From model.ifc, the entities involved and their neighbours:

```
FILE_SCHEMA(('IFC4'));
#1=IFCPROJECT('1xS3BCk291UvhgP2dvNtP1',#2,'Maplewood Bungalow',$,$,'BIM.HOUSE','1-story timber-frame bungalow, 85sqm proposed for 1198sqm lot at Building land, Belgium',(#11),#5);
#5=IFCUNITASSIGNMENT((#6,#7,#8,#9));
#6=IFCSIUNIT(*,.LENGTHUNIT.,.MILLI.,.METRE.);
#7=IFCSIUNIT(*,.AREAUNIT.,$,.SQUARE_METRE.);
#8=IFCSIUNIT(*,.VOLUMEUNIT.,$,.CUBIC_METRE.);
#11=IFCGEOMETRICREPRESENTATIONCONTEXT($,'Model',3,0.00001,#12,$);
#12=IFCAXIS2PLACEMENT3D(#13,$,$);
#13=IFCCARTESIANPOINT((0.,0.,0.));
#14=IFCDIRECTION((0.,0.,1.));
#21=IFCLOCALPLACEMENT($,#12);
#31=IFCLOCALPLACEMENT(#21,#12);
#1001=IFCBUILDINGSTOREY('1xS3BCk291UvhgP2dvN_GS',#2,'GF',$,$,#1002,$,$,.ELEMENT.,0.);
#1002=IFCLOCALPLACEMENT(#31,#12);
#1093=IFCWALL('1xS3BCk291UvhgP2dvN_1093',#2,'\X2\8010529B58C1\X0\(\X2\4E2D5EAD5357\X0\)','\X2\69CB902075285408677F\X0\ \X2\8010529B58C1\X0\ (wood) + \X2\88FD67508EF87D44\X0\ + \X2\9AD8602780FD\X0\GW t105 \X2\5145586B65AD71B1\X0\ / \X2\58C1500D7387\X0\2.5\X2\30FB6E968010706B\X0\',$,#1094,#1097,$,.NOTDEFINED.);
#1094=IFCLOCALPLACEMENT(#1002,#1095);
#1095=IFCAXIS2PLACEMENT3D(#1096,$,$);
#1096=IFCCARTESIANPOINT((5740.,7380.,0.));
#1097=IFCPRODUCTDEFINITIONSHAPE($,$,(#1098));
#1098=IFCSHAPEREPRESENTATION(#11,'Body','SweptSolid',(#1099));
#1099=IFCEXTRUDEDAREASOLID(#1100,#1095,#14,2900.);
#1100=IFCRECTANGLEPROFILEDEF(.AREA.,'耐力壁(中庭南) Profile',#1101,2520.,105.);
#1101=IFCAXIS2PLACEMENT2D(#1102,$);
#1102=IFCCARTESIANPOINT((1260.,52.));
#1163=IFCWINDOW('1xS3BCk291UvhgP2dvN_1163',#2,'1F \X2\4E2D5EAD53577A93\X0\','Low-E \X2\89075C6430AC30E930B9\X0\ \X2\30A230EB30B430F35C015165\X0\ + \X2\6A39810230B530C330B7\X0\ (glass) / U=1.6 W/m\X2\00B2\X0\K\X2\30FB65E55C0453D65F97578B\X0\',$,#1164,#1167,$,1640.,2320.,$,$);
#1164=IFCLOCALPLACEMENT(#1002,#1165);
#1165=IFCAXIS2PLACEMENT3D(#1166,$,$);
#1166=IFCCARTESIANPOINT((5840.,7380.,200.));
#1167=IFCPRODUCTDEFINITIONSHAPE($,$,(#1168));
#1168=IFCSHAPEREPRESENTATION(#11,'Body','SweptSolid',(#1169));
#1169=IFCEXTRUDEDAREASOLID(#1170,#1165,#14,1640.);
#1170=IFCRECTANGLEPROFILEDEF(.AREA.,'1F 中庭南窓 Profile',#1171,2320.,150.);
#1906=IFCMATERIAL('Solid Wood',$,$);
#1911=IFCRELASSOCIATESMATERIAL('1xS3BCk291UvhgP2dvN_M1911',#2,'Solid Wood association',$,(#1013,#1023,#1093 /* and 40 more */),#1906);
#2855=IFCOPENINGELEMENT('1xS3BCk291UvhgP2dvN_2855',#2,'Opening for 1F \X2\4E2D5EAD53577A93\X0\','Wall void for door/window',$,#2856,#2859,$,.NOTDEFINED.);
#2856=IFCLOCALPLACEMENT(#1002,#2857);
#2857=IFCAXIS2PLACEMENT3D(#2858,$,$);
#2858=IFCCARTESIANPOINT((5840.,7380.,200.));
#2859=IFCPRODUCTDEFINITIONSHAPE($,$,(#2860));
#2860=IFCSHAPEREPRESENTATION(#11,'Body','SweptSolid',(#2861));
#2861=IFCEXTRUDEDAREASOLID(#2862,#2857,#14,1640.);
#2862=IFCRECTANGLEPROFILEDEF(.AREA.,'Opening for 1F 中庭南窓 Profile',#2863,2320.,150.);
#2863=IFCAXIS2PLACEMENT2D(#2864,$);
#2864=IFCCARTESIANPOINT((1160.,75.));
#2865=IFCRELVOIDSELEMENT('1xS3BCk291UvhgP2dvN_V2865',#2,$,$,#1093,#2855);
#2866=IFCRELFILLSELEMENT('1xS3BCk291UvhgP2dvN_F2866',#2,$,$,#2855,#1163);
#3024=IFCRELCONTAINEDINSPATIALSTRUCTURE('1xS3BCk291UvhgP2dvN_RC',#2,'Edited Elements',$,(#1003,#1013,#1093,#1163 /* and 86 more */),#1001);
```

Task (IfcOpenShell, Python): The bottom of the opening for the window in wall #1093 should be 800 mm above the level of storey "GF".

```python
import numpy as np
import ifcopenshell
import ifcopenshell.api.geometry
import ifcopenshell.geom
import ifcopenshell.util.element
import ifcopenshell.util.placement
import ifcopenshell.util.shape
import ifcopenshell.util.unit

model = ifcopenshell.open("model.ifc")
unit_scale = ifcopenshell.util.unit.calculate_unit_scale(model)

window = model.by_guid("1xS3BCk291UvhgP2dvN_1163")
opening = window.FillsVoids[0].RelatingOpeningElement
storey = ifcopenshell.util.element.get_container(window, ifc_class="IfcBuildingStorey")
level = ifcopenshell.util.placement.get_local_placement(storey.ObjectPlacement)[2, 3]

# The opening's origin need not be at the sill, so measure its lowest point.
shape = ifcopenshell.geom.create_shape(ifcopenshell.geom.settings(), opening)
bottom = ifcopenshell.util.shape.get_shape_bottom_elevation(shape, shape.geometry) / unit_scale
dz = level + 0.8 / unit_scale - bottom

shift = np.array([0.0, 0.0, dz])
# The window is not placed relative to its opening, so move both.
for product in (opening, window):
    matrix = ifcopenshell.util.placement.get_local_placement(product.ObjectPlacement)
    matrix[:3, 3] += shift
    ifcopenshell.api.geometry.edit_object_placement(model, product=product, matrix=matrix, is_si=False)

print(f"moved by {dz * unit_scale:+.3f} m")

model.write("model_updated.ifc")
```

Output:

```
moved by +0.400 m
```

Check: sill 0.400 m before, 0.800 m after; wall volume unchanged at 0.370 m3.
